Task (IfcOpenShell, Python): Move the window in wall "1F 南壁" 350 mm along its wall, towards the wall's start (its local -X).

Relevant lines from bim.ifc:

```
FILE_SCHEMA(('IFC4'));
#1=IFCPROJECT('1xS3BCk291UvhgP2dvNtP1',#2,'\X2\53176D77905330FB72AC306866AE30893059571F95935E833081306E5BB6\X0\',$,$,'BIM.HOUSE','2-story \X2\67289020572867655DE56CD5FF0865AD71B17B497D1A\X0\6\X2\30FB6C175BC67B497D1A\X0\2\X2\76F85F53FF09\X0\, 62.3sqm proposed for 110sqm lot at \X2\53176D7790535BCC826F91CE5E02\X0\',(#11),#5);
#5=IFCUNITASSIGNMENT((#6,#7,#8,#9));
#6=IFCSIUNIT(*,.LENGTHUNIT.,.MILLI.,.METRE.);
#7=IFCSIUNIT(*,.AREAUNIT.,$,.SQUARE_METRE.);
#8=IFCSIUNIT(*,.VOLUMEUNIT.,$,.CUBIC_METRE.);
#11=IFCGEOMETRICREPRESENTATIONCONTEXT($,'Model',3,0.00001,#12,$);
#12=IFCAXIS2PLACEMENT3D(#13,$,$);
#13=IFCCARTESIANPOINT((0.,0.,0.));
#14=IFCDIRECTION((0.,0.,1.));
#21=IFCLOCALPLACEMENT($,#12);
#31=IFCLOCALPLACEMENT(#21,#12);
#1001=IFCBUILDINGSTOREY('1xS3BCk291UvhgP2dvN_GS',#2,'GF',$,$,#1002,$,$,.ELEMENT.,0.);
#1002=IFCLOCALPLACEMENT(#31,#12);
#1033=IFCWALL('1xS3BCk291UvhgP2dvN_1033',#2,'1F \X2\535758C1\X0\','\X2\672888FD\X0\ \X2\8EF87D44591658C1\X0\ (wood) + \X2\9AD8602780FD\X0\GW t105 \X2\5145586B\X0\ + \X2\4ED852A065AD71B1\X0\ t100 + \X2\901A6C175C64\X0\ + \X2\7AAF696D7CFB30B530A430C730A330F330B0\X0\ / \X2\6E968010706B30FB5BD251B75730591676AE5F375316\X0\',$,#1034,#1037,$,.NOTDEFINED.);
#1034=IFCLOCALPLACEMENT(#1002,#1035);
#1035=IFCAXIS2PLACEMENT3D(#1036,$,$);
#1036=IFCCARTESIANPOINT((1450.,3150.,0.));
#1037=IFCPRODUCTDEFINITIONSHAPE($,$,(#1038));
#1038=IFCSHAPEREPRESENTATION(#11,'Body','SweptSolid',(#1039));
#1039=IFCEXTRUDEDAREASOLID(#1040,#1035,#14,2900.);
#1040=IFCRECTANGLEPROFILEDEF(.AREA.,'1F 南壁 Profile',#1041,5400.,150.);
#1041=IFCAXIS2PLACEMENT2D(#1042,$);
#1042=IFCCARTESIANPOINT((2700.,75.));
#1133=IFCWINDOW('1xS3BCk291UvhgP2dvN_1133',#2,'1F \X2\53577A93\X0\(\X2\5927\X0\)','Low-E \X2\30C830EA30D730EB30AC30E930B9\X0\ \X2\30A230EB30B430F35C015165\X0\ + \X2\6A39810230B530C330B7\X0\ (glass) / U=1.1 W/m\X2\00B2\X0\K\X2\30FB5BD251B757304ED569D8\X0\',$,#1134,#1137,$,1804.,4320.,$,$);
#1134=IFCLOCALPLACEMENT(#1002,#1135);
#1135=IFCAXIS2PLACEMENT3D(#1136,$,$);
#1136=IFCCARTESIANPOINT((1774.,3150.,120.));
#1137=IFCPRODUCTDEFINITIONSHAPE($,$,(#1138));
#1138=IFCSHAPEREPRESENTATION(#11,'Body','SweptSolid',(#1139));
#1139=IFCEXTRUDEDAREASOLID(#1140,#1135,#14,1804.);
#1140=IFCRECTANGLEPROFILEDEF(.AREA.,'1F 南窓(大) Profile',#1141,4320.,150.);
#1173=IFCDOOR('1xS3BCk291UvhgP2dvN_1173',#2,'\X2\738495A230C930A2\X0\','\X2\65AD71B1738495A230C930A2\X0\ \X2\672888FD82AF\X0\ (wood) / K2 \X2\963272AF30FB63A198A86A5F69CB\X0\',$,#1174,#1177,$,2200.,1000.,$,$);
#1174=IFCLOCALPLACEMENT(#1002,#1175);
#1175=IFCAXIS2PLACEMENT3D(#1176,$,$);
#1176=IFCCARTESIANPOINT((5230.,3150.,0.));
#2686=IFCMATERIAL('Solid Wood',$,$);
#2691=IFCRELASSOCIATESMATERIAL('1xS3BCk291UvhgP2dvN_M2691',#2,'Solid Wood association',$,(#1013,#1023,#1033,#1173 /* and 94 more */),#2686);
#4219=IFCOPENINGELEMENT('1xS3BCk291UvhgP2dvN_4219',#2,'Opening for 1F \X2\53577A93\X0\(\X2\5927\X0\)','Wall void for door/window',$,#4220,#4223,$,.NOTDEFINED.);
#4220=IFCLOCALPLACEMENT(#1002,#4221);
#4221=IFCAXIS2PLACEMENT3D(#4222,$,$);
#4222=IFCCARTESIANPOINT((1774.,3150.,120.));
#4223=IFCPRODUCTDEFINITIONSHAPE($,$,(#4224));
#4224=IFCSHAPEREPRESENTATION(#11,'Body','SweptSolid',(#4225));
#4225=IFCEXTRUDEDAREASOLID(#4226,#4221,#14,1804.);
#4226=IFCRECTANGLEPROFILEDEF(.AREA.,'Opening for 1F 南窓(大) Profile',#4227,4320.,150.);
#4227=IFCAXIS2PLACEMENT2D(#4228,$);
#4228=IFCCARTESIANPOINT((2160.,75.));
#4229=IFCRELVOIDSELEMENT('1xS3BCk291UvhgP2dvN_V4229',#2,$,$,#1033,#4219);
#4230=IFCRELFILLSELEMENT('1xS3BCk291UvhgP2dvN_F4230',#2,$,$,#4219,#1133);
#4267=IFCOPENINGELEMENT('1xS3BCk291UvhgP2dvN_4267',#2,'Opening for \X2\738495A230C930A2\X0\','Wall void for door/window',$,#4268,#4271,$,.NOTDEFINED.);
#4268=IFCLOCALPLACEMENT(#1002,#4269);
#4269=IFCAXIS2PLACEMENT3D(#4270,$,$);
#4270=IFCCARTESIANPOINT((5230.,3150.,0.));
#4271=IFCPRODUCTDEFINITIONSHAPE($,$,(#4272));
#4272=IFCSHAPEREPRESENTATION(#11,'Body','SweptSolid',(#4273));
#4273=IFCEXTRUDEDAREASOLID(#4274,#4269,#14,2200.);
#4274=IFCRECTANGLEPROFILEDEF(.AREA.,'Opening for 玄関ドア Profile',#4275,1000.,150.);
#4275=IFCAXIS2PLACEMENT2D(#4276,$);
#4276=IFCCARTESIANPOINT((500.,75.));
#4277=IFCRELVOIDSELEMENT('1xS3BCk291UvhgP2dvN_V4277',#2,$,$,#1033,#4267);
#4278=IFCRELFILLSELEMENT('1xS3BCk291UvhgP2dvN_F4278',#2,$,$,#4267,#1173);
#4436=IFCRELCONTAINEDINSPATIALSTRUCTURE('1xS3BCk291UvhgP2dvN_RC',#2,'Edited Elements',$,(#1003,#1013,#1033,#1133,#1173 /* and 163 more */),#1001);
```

```python
import ifcopenshell
import ifcopenshell.api.geometry
import ifcopenshell.util.placement

model = ifcopenshell.open("bim.ifc")

window = model.by_guid("1xS3BCk291UvhgP2dvN_1133")
opening = window.FillsVoids[0].RelatingOpeningElement
wall = opening.VoidsElements[0].RelatingBuildingElement

wall_matrix = ifcopenshell.util.placement.get_local_placement(wall.ObjectPlacement)
shift = wall_matrix[:3, 0] * -350.0
before = ifcopenshell.util.placement.get_local_placement(window.ObjectPlacement)[:3, 3].copy()

# The window is not placed relative to its opening, so move both.
for product in (opening, window):
    matrix = ifcopenshell.util.placement.get_local_placement(product.ObjectPlacement)
    matrix[:3, 3] += shift
    ifcopenshell.api.geometry.edit_object_placement(model, product=product, matrix=matrix, is_si=False)

after = ifcopenshell.util.placement.get_local_placement(window.ObjectPlacement)[:3, 3]
print("window moved by", (after - before).round(3) + 0.0)

model.write("bim_v2.ifc")
```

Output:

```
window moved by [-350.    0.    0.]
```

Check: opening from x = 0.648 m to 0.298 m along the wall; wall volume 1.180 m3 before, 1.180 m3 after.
